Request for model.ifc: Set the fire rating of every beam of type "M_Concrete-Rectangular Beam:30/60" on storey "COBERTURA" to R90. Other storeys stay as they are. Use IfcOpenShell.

First a look at what the model holds.

```python
import ifcopenshell
import ifcopenshell.util.element

model = ifcopenshell.open("model.ifc")
print(model.schema)
storey = next(s for s in model.by_type("IfcBuildingStorey") if s.Name == "COBERTURA")
beams = [e for e in ifcopenshell.util.element.get_decomposition(storey) if e.is_a("IfcBeam")]
seen = {}
for e in beams:
    element_type = ifcopenshell.util.element.get_type(e)
    key = (element_type.Name if element_type != e and element_type else None, ifcopenshell.util.element.get_pset(e, "Pset_BeamCommon", "FireRating"))
    seen[key] = seen.get(key, 0) + 1
for (name, value), count in sorted(seen.items(), key=str):
    print(count, "x", name, "|", value)
```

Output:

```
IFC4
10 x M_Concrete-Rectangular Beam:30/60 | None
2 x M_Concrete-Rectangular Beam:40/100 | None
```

```python
import ifcopenshell
import ifcopenshell.api.pset
import ifcopenshell.util.element

model = ifcopenshell.open("model.ifc")

storey = next(s for s in model.by_type("IfcBuildingStorey") if s.Name == "COBERTURA")
beams = [e for e in ifcopenshell.util.element.get_decomposition(storey) if e.is_a("IfcBeam")]

count = 0
for e in beams:
    element_type = ifcopenshell.util.element.get_type(e)
    if element_type in (None, e) or element_type.Name != "M_Concrete-Rectangular Beam:30/60":
        continue
    # add_pset returns the element's existing set when there is one.
    pset = ifcopenshell.api.pset.add_pset(model, product=e, name="Pset_BeamCommon")
    ifcopenshell.api.pset.edit_pset(model, pset=pset, properties={"FireRating": "R90"})
    count += 1

print(count, "beams updated")

model.write("model_v2.ifc")
```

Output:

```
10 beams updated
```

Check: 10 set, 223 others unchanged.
